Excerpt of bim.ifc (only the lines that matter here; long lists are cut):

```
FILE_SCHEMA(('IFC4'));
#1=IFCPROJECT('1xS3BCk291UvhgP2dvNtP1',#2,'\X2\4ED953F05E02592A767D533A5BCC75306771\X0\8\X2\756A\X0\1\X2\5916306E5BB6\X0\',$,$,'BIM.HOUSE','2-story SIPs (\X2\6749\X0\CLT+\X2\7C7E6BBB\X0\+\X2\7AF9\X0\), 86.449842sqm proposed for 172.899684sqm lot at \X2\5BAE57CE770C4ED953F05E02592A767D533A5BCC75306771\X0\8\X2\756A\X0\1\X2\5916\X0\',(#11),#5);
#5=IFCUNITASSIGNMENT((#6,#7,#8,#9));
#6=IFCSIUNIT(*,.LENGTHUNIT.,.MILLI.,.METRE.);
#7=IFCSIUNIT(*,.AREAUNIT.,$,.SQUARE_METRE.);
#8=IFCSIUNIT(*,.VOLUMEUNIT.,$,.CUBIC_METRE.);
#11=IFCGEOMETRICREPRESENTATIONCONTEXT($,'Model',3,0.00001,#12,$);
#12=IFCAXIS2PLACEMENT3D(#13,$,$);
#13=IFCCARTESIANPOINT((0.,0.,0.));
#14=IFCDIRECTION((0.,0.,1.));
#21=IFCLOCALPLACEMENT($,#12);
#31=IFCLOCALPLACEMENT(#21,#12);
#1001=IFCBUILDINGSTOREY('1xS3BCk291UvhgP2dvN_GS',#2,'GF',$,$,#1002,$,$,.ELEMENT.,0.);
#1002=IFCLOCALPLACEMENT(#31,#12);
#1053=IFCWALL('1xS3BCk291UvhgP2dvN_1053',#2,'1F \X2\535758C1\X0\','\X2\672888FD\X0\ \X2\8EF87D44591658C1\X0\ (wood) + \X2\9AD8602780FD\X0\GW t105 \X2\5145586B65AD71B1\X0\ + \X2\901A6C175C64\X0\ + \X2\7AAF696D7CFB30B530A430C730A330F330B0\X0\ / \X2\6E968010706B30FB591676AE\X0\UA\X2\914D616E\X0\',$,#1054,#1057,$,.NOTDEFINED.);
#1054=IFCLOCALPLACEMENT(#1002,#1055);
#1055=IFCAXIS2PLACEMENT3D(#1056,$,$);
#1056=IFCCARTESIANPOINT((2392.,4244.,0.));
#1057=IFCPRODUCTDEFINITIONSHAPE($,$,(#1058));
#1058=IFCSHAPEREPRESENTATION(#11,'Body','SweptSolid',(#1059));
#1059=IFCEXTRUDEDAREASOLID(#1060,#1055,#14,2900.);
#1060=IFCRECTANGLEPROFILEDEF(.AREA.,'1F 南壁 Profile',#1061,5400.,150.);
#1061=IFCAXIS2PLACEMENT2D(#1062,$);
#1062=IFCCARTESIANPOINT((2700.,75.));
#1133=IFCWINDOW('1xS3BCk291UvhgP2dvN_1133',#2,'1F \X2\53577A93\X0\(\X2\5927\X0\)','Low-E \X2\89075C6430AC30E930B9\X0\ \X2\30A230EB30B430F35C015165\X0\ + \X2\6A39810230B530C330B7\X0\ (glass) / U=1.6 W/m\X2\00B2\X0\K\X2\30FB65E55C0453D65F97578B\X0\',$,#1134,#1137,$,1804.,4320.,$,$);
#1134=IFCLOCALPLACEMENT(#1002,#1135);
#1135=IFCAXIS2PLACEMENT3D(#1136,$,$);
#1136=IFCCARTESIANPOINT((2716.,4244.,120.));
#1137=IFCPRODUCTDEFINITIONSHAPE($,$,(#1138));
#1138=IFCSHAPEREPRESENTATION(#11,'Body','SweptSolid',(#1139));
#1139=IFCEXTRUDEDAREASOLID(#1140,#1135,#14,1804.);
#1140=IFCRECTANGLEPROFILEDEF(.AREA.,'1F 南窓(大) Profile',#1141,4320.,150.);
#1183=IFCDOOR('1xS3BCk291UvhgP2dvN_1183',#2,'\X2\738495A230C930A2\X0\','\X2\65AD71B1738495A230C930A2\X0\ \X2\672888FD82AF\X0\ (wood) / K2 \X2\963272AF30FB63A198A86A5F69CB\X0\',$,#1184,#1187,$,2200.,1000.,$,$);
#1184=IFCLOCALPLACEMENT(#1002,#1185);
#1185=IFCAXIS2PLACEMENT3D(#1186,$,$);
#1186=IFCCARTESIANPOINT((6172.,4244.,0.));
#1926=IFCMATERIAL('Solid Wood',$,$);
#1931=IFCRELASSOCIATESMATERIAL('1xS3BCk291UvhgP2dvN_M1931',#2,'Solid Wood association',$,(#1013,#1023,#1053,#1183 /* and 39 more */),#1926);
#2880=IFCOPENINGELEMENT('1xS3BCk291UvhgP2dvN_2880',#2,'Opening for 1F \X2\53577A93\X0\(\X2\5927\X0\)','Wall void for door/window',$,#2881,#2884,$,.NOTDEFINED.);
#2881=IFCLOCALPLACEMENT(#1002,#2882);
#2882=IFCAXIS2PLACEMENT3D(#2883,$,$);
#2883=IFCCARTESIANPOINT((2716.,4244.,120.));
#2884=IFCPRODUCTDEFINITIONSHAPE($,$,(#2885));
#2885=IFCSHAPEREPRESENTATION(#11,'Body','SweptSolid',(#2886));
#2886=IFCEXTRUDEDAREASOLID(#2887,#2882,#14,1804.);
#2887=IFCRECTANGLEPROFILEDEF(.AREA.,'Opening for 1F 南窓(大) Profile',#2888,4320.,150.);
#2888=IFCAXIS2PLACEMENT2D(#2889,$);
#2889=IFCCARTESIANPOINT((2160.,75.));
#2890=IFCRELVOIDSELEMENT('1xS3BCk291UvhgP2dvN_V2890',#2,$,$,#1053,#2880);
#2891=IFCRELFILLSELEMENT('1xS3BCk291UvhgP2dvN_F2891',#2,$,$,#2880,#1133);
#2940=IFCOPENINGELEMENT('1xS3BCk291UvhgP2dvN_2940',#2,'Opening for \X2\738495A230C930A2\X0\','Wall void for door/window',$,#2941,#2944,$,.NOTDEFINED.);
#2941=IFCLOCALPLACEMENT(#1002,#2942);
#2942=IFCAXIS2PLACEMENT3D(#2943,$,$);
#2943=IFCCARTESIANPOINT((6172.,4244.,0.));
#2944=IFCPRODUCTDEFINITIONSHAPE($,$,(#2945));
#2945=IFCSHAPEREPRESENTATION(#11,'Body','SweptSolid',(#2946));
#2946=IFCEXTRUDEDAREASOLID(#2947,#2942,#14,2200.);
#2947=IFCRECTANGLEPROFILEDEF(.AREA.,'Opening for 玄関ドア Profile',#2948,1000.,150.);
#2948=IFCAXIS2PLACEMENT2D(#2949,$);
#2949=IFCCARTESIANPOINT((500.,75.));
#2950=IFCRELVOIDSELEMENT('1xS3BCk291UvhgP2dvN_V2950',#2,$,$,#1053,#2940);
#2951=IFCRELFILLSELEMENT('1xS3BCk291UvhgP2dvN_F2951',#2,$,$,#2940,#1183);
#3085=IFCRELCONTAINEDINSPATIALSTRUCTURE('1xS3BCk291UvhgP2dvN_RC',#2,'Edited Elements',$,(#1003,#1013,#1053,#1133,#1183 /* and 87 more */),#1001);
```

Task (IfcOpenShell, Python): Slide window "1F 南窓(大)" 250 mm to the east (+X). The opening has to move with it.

```python
import ifcopenshell
import ifcopenshell.api.geometry
import ifcopenshell.util.placement

model = ifcopenshell.open("bim.ifc")

window = model.by_guid("1xS3BCk291UvhgP2dvN_1133")
opening = window.FillsVoids[0].RelatingOpeningElement
wall = opening.VoidsElements[0].RelatingBuildingElement

wall_matrix = ifcopenshell.util.placement.get_local_placement(wall.ObjectPlacement)
shift = wall_matrix[:3, 0] * 250.0
before = ifcopenshell.util.placement.get_local_placement(window.ObjectPlacement)[:3, 3].copy()

# The window is not placed relative to its opening, so move both.
for product in (opening, window):
    matrix = ifcopenshell.util.placement.get_local_placement(product.ObjectPlacement)
    matrix[:3, 3] += shift
    ifcopenshell.api.geometry.edit_object_placement(model, product=product, matrix=matrix, is_si=False)

after = ifcopenshell.util.placement.get_local_placement(window.ObjectPlacement)[:3, 3]
print("window moved by", (after - before).round(3) + 0.0)

model.write("bim_rev.ifc")
```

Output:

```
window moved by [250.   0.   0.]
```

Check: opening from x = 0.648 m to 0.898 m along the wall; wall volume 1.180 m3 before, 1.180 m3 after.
